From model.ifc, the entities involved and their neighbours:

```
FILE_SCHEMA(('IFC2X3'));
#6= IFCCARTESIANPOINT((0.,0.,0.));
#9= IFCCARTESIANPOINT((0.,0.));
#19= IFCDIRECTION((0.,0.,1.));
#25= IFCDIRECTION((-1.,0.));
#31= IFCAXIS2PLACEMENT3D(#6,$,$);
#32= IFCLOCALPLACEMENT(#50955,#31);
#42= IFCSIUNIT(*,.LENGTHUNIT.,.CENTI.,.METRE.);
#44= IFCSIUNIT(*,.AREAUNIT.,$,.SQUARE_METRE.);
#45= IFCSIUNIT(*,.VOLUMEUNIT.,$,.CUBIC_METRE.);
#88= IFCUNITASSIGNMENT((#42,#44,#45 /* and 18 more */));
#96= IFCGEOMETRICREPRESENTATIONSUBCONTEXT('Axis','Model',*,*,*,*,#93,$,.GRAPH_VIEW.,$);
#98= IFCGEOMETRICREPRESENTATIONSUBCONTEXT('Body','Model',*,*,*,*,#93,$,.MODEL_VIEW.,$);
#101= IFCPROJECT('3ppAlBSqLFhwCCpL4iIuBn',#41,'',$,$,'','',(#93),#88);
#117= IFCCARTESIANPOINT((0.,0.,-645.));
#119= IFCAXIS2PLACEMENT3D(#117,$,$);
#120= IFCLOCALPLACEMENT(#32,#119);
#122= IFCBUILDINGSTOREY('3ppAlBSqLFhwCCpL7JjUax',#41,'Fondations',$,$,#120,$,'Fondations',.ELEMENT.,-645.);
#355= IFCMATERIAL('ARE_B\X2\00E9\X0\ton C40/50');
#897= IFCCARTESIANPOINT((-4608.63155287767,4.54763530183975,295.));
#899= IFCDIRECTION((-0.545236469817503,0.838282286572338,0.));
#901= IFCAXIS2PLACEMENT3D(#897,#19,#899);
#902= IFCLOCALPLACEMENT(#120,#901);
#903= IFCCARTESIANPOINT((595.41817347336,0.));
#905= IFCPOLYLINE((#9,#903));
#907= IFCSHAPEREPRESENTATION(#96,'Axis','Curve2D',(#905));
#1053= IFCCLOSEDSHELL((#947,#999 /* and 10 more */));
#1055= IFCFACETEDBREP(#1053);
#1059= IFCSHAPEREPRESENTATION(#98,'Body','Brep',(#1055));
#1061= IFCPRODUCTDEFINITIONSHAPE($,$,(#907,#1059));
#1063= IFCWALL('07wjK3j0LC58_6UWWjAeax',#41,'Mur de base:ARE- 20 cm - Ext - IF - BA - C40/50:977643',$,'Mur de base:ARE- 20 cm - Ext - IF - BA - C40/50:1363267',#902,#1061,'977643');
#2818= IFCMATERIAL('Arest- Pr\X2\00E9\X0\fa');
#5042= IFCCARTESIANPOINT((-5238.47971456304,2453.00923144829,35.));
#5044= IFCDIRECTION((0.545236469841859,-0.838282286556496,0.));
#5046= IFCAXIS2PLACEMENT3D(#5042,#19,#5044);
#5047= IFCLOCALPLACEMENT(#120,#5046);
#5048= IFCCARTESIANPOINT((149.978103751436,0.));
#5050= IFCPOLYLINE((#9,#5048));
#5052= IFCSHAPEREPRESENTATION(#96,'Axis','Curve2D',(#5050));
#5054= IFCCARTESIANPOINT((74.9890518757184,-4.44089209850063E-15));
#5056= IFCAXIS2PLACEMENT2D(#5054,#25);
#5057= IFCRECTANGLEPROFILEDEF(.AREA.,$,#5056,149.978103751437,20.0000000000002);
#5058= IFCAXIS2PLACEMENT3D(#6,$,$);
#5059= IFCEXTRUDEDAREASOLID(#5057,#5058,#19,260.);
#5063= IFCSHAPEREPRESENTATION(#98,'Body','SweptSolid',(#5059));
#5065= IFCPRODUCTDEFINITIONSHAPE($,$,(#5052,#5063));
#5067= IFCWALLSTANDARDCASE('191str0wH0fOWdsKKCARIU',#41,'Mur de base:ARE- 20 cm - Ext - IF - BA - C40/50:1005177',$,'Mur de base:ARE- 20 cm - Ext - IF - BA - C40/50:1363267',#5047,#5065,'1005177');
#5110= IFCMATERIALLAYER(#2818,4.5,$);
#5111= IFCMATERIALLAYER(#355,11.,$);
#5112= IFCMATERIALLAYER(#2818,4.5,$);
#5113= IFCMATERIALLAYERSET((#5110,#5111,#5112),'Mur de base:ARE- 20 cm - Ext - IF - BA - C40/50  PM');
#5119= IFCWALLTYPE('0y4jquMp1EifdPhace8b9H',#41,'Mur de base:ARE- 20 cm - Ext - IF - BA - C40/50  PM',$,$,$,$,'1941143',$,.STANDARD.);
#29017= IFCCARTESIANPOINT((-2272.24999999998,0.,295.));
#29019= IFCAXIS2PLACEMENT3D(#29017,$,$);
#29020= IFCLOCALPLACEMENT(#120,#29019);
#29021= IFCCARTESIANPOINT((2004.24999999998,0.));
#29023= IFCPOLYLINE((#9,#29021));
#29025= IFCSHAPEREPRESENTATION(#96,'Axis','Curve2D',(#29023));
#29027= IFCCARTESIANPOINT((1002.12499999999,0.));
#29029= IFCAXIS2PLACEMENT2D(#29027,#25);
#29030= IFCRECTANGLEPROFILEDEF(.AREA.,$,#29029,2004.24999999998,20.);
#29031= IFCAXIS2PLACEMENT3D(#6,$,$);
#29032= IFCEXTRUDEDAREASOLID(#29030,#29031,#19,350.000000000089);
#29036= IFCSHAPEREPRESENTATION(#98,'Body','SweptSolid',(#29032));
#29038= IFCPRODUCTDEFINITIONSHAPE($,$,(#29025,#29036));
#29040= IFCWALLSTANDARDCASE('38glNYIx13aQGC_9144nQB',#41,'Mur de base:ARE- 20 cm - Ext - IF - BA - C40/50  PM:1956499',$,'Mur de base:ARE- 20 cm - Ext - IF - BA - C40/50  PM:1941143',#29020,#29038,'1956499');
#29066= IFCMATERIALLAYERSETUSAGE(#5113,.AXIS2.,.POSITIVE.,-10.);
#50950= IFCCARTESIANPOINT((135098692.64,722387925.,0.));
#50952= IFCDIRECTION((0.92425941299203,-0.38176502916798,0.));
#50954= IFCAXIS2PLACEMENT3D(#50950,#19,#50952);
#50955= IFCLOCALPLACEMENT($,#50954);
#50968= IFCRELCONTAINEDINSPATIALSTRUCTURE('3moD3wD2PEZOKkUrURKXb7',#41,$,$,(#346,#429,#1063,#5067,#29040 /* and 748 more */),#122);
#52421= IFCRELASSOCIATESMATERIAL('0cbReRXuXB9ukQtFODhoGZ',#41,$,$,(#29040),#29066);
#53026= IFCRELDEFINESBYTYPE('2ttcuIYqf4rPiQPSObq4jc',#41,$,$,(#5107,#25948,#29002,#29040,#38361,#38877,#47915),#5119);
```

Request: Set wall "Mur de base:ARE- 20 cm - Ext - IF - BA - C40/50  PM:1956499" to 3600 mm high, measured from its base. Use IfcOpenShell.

```python
import ifcopenshell
import ifcopenshell.geom
import ifcopenshell.util.representation
import ifcopenshell.util.shape
import ifcopenshell.util.unit

model = ifcopenshell.open("model.ifc")
unit_scale = ifcopenshell.util.unit.calculate_unit_scale(model)
settings = ifcopenshell.geom.settings()


def volume(element):
    """Net volume in cubic metres, openings subtracted."""
    shape = ifcopenshell.geom.create_shape(settings, element)
    return ifcopenshell.util.shape.get_volume(shape.geometry)


wall = model.by_guid("38glNYIx13aQGC_9144nQB")
before = volume(wall)

body = ifcopenshell.util.representation.get_representation(wall, "Model", "Body")
solid = body.Items[0]
old_height = solid.Depth
solid.Depth = 3.6 / unit_scale
after = volume(wall)

print(f"height {old_height:g} -> {solid.Depth:g}, volume {before:.3f} -> {after:.3f} m3")

model.write("model_v2.ifc")
```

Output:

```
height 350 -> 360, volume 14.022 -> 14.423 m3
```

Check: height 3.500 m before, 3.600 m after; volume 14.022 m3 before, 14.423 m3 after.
